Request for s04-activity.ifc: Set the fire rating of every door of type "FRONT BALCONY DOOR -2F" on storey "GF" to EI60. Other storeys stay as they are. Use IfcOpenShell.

First a look at what the model holds.

```python
import ifcopenshell
import ifcopenshell.util.element

model = ifcopenshell.open("s04-activity.ifc")
print(model.schema)
storey = next(s for s in model.by_type("IfcBuildingStorey") if s.Name == "GF")
doors = [e for e in ifcopenshell.util.element.get_decomposition(storey) if e.is_a("IfcDoor")]
seen = {}
for e in doors:
    element_type = ifcopenshell.util.element.get_type(e)
    key = (element_type.Name if element_type != e and element_type else None, ifcopenshell.util.element.get_pset(e, "Pset_DoorCommon", "FireRating"))
    seen[key] = seen.get(key, 0) + 1
for (name, value), count in sorted(seen.items(), key=str):
    print(count, "x", name, "|", value)
```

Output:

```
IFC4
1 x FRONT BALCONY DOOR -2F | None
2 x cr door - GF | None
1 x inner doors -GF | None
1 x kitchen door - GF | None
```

```python
import ifcopenshell
import ifcopenshell.api.pset
import ifcopenshell.util.element

model = ifcopenshell.open("s04-activity.ifc")

storey = next(s for s in model.by_type("IfcBuildingStorey") if s.Name == "GF")
doors = [e for e in ifcopenshell.util.element.get_decomposition(storey) if e.is_a("IfcDoor")]

count = 0
for e in doors:
    element_type = ifcopenshell.util.element.get_type(e)
    if element_type in (None, e) or element_type.Name != "FRONT BALCONY DOOR -2F":
        continue
    # add_pset returns the element's existing set when there is one.
    pset = ifcopenshell.api.pset.add_pset(model, product=e, name="Pset_DoorCommon")
    ifcopenshell.api.pset.edit_pset(model, pset=pset, properties={"FireRating": "EI60"})
    count += 1

print(count, "doors updated")

model.write("s04-activity_edited.ifc")
```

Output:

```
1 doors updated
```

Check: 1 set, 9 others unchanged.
